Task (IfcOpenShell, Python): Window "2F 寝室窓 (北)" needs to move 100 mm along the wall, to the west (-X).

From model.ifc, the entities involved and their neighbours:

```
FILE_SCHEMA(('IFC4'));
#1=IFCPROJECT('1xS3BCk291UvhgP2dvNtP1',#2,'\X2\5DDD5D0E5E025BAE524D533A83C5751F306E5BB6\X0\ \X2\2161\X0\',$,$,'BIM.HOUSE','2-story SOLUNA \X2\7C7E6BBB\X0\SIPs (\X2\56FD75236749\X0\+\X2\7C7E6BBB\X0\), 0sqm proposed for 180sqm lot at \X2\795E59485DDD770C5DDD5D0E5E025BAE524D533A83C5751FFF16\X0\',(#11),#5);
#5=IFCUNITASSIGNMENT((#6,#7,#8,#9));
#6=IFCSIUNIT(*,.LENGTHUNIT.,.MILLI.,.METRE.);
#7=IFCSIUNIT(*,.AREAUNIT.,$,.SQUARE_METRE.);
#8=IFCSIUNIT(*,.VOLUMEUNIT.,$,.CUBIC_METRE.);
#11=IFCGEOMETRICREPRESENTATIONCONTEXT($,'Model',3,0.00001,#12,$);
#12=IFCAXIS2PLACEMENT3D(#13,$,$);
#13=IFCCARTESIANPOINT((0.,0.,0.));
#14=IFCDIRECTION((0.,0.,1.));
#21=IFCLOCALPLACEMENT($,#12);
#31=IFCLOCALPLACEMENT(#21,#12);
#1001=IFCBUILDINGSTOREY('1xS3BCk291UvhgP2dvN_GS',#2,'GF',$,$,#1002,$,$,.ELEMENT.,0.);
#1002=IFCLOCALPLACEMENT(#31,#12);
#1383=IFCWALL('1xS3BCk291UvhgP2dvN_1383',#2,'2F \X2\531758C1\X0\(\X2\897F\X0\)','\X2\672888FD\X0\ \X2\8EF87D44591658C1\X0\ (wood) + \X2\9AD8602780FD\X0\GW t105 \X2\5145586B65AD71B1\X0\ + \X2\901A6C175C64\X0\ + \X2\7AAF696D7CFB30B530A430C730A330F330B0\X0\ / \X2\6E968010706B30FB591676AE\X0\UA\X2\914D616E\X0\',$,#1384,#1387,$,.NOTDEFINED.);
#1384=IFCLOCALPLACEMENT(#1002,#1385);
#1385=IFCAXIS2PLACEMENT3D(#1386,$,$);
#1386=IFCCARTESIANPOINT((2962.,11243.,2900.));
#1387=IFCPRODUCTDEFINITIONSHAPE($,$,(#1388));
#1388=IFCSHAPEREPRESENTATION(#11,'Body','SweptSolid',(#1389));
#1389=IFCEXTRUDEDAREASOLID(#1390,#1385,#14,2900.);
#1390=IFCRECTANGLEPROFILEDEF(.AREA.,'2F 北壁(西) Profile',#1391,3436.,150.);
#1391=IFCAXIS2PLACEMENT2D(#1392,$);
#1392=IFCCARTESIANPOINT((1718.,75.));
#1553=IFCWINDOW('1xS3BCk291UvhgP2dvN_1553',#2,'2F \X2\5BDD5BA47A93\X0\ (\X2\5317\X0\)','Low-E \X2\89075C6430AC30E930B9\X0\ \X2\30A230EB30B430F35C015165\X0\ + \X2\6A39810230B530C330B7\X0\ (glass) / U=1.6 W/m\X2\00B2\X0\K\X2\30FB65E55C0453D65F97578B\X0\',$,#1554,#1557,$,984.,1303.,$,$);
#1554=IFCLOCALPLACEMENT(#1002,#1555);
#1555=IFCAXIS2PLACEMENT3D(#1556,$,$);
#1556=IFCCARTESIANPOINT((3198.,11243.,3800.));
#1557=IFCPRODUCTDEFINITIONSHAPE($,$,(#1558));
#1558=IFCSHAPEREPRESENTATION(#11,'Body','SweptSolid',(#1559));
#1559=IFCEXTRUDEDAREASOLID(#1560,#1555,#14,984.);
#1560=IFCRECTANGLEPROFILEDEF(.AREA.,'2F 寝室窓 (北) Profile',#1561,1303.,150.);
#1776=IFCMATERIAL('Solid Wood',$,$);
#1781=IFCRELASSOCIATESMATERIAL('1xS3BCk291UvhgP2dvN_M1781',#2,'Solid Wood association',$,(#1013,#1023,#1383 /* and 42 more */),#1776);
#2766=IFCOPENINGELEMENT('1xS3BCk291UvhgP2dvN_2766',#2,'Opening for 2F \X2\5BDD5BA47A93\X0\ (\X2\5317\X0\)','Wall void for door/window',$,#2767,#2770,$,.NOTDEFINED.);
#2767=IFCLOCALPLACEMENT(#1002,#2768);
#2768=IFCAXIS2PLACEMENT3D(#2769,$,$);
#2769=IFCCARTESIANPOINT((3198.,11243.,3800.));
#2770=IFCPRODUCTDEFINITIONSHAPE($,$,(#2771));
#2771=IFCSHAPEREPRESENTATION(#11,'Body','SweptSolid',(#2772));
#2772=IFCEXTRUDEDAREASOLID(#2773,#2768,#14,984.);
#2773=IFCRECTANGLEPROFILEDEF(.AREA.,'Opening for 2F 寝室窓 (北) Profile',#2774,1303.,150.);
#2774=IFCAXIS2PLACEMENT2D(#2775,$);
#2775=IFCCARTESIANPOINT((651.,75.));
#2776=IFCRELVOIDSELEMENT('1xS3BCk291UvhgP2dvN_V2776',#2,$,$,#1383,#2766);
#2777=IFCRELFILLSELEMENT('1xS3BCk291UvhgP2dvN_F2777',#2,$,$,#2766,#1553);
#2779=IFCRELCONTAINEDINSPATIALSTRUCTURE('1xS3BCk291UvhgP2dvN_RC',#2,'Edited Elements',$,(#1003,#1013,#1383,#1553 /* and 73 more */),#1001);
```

```python
import ifcopenshell
import ifcopenshell.api.geometry
import ifcopenshell.util.placement
import ifcopenshell.util.unit

model = ifcopenshell.open("model.ifc")
unit_scale = ifcopenshell.util.unit.calculate_unit_scale(model)

window = model.by_id(1553)
opening = window.FillsVoids[0].RelatingOpeningElement
wall = opening.VoidsElements[0].RelatingBuildingElement

wall_matrix = ifcopenshell.util.placement.get_local_placement(wall.ObjectPlacement)
shift = wall_matrix[:3, 0] * -0.1 / unit_scale
before = ifcopenshell.util.placement.get_local_placement(window.ObjectPlacement)[:3, 3].copy()

# The window is not placed relative to its opening, so move both.
for product in (opening, window):
    matrix = ifcopenshell.util.placement.get_local_placement(product.ObjectPlacement)
    matrix[:3, 3] += shift
    ifcopenshell.api.geometry.edit_object_placement(model, product=product, matrix=matrix, is_si=False)

after = ifcopenshell.util.placement.get_local_placement(window.ObjectPlacement)[:3, 3]
print("window moved by", (after - before).round(3) + 0.0)

model.write("model_v2.ifc")
```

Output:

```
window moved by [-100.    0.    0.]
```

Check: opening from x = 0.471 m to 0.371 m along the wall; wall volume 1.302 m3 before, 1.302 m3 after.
